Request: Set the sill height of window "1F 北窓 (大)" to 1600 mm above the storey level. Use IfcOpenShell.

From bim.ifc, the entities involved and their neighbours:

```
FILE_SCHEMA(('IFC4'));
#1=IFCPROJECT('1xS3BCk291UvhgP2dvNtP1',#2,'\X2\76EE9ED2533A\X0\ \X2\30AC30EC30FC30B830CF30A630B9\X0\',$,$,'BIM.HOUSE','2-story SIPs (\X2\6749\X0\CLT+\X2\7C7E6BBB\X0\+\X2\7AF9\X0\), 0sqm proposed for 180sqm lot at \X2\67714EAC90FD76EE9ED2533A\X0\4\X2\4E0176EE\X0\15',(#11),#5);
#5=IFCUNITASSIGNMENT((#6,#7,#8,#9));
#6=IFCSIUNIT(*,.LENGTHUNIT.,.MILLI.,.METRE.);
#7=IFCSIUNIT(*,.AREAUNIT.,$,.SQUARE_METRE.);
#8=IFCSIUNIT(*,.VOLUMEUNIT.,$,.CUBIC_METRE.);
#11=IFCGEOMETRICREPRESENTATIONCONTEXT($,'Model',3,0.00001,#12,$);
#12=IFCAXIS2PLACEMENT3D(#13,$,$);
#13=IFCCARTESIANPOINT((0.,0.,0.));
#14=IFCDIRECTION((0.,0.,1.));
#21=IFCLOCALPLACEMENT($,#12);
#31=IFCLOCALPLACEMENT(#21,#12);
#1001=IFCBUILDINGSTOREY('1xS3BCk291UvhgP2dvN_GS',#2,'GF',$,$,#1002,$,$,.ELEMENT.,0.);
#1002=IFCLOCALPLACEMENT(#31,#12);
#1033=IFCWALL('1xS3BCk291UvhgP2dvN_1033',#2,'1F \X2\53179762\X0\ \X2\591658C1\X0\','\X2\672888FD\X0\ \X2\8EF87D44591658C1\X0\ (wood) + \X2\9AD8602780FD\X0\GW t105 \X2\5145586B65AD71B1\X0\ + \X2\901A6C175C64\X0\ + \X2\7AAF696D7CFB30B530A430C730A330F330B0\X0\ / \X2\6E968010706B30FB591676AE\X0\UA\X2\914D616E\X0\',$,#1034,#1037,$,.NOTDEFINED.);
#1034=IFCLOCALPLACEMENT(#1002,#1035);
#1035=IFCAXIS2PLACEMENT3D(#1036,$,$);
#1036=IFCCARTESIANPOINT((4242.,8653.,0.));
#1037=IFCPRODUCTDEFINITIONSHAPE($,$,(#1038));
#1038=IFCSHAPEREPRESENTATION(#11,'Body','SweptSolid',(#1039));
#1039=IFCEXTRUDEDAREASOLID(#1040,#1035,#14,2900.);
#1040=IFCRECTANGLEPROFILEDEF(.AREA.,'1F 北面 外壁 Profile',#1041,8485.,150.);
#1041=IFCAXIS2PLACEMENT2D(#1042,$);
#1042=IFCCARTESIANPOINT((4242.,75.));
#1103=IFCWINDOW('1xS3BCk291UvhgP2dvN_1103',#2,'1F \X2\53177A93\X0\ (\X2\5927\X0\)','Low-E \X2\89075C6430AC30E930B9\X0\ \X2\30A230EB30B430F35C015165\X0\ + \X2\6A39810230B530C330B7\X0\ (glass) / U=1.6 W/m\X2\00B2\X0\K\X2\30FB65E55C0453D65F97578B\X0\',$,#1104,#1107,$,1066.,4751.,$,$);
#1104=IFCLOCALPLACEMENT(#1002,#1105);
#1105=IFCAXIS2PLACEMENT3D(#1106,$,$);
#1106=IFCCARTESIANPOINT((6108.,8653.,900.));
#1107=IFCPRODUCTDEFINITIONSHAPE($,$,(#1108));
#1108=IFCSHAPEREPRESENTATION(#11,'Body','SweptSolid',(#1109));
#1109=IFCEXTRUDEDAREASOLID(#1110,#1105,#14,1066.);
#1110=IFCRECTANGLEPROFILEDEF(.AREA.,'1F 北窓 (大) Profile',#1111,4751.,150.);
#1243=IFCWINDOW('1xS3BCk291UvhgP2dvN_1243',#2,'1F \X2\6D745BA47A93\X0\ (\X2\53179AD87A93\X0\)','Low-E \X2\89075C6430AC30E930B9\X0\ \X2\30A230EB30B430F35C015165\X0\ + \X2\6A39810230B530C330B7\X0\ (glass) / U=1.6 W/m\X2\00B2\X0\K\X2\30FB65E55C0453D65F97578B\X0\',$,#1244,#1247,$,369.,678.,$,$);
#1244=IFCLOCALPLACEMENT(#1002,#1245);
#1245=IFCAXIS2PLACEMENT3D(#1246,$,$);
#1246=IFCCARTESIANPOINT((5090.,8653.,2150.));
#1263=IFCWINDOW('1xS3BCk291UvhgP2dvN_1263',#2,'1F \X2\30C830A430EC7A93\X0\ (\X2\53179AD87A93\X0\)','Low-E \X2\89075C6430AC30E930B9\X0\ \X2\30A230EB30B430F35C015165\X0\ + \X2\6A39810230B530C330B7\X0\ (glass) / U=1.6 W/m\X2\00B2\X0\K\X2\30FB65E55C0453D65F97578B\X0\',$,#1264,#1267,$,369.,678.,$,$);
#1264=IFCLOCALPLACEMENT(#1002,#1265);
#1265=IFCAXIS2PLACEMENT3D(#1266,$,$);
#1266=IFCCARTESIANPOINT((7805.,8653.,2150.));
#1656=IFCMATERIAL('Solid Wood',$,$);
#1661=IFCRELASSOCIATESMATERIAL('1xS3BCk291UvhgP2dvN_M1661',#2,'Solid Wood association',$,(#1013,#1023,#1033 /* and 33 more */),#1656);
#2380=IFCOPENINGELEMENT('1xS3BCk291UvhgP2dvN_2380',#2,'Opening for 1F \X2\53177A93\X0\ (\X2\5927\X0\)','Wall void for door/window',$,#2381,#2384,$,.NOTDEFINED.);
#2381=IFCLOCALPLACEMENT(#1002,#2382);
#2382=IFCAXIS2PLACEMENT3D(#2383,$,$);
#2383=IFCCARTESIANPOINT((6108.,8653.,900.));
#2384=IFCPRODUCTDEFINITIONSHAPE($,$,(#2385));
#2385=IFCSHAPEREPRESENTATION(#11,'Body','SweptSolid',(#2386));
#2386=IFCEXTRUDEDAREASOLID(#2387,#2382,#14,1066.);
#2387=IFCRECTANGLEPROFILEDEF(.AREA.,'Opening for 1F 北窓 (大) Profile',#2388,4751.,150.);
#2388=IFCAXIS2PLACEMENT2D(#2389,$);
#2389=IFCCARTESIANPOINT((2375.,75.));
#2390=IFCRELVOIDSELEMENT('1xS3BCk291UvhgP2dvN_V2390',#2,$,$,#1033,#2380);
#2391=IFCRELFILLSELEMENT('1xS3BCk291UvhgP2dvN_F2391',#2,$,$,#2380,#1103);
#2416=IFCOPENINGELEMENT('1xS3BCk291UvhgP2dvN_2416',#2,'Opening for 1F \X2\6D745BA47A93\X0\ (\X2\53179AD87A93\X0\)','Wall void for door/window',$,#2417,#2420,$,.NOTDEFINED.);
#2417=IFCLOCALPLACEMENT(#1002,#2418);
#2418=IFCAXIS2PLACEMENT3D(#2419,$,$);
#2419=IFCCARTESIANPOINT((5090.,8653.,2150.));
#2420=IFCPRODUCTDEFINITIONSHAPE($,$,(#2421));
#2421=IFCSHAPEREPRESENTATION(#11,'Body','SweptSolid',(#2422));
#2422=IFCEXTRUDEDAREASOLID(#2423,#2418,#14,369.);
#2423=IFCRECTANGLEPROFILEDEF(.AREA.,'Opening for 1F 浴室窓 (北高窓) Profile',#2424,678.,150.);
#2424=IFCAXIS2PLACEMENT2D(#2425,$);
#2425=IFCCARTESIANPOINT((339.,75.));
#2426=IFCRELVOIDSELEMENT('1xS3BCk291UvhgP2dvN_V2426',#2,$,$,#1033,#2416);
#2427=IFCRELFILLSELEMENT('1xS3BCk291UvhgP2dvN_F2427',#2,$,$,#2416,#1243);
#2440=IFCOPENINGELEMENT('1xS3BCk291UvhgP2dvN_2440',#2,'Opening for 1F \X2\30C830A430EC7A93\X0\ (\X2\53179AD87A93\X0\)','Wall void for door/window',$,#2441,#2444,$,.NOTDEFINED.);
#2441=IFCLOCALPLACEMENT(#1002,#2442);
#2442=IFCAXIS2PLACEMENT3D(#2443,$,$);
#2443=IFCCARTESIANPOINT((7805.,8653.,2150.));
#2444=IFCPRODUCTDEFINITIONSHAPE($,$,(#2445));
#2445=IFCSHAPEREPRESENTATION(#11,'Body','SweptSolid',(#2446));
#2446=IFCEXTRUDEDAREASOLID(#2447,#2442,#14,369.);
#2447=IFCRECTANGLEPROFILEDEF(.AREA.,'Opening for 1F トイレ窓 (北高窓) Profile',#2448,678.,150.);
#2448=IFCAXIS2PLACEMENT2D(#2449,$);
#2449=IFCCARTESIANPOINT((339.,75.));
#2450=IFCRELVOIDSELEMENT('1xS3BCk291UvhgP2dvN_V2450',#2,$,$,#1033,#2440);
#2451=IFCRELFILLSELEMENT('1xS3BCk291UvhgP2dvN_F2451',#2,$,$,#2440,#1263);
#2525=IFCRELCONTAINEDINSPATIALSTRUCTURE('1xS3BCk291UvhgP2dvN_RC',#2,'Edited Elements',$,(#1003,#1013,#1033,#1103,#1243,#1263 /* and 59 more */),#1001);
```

```python
import numpy as np
import ifcopenshell
import ifcopenshell.api.geometry
import ifcopenshell.geom
import ifcopenshell.util.element
import ifcopenshell.util.placement
import ifcopenshell.util.shape
import ifcopenshell.util.unit

model = ifcopenshell.open("bim.ifc")
unit_scale = ifcopenshell.util.unit.calculate_unit_scale(model)

window = model.by_guid("1xS3BCk291UvhgP2dvN_1103")
opening = window.FillsVoids[0].RelatingOpeningElement
storey = ifcopenshell.util.element.get_container(window, ifc_class="IfcBuildingStorey")
level = ifcopenshell.util.placement.get_local_placement(storey.ObjectPlacement)[2, 3]

# The opening's origin need not be at the sill, so measure its lowest point.
shape = ifcopenshell.geom.create_shape(ifcopenshell.geom.settings(), opening)
bottom = ifcopenshell.util.shape.get_shape_bottom_elevation(shape, shape.geometry) / unit_scale
dz = level + 1.6 / unit_scale - bottom

shift = np.array([0.0, 0.0, dz])
# The window is not placed relative to its opening, so move both.
for product in (opening, window):
    matrix = ifcopenshell.util.placement.get_local_placement(product.ObjectPlacement)
    matrix[:3, 3] += shift
    ifcopenshell.api.geometry.edit_object_placement(model, product=product, matrix=matrix, is_si=False)

print(f"moved by {dz * unit_scale:+.3f} m")

model.write("bim_edited.ifc")
```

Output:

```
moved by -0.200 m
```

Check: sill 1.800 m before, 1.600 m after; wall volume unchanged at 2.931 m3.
